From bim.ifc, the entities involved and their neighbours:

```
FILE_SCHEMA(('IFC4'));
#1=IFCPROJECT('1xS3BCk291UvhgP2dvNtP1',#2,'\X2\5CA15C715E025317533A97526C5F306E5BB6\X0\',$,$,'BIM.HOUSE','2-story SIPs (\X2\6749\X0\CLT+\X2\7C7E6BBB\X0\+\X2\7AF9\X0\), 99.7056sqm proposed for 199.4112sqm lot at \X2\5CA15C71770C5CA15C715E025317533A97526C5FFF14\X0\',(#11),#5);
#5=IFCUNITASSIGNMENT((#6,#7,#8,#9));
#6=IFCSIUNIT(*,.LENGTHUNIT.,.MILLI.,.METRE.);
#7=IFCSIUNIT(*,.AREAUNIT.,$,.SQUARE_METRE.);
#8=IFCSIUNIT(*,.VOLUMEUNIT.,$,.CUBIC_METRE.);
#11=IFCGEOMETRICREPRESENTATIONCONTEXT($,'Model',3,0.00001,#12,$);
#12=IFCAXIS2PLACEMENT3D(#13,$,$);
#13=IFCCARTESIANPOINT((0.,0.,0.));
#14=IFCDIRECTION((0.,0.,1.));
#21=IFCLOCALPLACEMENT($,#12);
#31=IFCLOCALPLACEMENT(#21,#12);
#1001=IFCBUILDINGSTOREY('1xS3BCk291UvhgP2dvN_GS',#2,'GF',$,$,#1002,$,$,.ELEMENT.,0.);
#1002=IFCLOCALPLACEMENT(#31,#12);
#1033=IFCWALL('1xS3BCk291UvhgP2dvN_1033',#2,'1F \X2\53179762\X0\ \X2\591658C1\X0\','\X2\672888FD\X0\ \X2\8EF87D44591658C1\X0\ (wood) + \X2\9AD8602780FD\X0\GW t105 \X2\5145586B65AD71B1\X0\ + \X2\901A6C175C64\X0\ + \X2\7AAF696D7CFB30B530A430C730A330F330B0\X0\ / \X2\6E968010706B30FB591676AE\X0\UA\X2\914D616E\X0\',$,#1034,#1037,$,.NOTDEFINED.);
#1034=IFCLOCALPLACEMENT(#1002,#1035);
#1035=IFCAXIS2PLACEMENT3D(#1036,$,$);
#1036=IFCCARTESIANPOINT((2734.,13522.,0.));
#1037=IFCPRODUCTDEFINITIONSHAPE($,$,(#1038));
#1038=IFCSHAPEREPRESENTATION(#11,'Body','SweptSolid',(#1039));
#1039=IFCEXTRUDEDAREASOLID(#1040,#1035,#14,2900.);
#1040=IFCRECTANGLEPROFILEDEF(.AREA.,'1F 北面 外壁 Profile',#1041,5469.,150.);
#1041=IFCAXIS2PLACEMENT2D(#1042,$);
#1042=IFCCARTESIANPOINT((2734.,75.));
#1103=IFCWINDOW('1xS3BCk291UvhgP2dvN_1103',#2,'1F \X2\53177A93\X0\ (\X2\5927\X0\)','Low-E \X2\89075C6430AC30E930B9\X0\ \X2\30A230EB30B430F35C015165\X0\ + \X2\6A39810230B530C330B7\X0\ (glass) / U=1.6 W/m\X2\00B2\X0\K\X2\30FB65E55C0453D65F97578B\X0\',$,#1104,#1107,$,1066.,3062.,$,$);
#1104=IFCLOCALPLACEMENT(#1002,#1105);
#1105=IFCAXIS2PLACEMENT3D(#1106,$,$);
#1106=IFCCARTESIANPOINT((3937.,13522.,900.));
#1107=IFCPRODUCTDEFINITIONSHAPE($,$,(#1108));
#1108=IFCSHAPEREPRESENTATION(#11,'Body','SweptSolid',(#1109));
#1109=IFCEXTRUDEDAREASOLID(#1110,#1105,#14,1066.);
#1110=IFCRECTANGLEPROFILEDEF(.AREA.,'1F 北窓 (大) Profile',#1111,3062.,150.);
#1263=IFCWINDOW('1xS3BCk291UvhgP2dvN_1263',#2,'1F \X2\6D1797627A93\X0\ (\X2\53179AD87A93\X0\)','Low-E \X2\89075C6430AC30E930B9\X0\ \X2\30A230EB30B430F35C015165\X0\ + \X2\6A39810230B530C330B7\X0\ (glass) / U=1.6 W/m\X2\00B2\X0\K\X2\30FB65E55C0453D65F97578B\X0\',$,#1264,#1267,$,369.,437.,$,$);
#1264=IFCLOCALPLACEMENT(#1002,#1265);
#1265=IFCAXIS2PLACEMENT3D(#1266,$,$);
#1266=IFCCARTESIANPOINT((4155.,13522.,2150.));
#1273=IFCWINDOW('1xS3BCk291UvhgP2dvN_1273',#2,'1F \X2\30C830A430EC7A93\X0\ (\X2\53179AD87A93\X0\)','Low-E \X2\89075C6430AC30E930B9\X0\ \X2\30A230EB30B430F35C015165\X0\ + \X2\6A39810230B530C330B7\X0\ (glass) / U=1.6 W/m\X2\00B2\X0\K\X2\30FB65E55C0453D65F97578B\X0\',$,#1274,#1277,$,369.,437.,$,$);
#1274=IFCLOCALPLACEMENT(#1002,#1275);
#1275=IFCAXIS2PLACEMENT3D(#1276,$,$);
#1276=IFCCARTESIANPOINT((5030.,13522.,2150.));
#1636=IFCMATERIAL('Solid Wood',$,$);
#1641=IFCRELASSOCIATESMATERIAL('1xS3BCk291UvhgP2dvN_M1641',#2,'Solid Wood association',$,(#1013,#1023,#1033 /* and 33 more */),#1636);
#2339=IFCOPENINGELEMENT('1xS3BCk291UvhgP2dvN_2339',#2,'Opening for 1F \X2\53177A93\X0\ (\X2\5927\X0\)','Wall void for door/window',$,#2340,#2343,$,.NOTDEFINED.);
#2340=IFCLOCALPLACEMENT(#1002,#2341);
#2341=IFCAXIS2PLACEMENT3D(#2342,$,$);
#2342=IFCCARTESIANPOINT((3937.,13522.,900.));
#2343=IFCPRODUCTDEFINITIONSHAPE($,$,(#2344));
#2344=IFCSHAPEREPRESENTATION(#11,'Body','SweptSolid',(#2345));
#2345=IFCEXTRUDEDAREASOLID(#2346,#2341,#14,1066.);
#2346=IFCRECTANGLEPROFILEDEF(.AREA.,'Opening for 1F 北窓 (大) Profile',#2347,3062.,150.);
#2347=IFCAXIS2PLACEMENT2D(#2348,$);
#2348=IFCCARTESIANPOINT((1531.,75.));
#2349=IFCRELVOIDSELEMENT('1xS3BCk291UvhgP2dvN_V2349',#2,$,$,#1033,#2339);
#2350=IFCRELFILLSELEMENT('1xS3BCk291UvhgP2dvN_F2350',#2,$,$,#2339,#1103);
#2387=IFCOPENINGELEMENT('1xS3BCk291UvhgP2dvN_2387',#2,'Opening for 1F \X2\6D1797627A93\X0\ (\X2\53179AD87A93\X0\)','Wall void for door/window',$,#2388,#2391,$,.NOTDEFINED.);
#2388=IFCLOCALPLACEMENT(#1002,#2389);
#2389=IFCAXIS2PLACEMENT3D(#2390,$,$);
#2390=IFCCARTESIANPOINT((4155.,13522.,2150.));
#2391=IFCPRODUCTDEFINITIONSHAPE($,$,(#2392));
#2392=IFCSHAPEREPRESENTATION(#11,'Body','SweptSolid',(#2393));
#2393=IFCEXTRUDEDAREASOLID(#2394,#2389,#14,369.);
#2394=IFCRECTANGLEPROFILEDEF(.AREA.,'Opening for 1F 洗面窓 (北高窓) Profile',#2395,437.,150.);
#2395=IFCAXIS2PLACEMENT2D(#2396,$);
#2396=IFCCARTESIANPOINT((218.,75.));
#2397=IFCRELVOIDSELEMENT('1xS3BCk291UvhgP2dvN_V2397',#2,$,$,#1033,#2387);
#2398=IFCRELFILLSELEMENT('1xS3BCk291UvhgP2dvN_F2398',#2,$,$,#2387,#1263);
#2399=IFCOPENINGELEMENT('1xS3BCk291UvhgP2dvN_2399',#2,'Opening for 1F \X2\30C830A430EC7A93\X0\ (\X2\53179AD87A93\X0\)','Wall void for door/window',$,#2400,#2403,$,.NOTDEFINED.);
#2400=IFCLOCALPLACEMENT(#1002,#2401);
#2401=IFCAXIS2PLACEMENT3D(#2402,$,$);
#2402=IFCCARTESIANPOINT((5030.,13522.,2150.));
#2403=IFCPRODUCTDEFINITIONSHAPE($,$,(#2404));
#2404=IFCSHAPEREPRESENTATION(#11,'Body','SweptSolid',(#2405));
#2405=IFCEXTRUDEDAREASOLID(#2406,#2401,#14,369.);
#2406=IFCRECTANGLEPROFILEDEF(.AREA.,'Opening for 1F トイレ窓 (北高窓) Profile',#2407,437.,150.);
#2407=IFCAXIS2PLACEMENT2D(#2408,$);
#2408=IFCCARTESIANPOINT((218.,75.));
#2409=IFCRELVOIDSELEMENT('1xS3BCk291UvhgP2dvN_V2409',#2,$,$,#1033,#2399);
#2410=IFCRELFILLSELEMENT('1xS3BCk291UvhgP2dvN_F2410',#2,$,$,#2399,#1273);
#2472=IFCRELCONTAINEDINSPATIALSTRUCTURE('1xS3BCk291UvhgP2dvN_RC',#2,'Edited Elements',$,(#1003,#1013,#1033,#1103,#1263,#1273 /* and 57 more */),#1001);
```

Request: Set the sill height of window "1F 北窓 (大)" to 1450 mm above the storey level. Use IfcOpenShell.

```python
import numpy as np
import ifcopenshell
import ifcopenshell.api.geometry
import ifcopenshell.geom
import ifcopenshell.util.element
import ifcopenshell.util.placement
import ifcopenshell.util.shape
import ifcopenshell.util.unit

model = ifcopenshell.open("bim.ifc")
unit_scale = ifcopenshell.util.unit.calculate_unit_scale(model)

window = model.by_id(1103)
opening = window.FillsVoids[0].RelatingOpeningElement
storey = ifcopenshell.util.element.get_container(window, ifc_class="IfcBuildingStorey")
level = ifcopenshell.util.placement.get_local_placement(storey.ObjectPlacement)[2, 3]

# The opening's origin need not be at the sill, so measure its lowest point.
shape = ifcopenshell.geom.create_shape(ifcopenshell.geom.settings(), opening)
bottom = ifcopenshell.util.shape.get_shape_bottom_elevation(shape, shape.geometry) / unit_scale
dz = level + 1.45 / unit_scale - bottom

shift = np.array([0.0, 0.0, dz])
# The window is not placed relative to its opening, so move both.
for product in (opening, window):
    matrix = ifcopenshell.util.placement.get_local_placement(product.ObjectPlacement)
    matrix[:3, 3] += shift
    ifcopenshell.api.geometry.edit_object_placement(model, product=product, matrix=matrix, is_si=False)

print(f"moved by {dz * unit_scale:+.3f} m")

model.write("bim_v2.ifc")
```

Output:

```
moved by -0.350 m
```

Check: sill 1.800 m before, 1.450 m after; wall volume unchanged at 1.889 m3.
